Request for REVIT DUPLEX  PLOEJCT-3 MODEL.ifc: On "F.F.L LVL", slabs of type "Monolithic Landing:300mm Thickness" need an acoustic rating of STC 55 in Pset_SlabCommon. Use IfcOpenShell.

First a look at what the model holds.

```python
import ifcopenshell
import ifcopenshell.util.element

model = ifcopenshell.open("REVIT DUPLEX  PLOEJCT-3 MODEL.ifc")
print(model.schema)
storey = next(s for s in model.by_type("IfcBuildingStorey") if s.Name == "F.F.L LVL")
slabs = [e for e in ifcopenshell.util.element.get_decomposition(storey) if e.is_a("IfcSlab")]
seen = {}
for e in slabs:
    element_type = ifcopenshell.util.element.get_type(e)
    key = (element_type.Name if element_type != e and element_type else None, ifcopenshell.util.element.get_pset(e, "Pset_SlabCommon", "AcousticRating"))
    seen[key] = seen.get(key, 0) + 1
for (name, value), count in sorted(seen.items(), key=str):
    print(count, "x", name, "|", value)
```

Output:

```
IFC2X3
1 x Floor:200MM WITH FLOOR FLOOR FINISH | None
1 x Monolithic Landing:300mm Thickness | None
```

```python
import ifcopenshell
import ifcopenshell.api.pset
import ifcopenshell.util.element

model = ifcopenshell.open("REVIT DUPLEX  PLOEJCT-3 MODEL.ifc")

storey = next(s for s in model.by_type("IfcBuildingStorey") if s.Name == "F.F.L LVL")
slabs = [e for e in ifcopenshell.util.element.get_decomposition(storey) if e.is_a("IfcSlab")]

count = 0
for e in slabs:
    element_type = ifcopenshell.util.element.get_type(e)
    if element_type in (None, e) or element_type.Name != "Monolithic Landing:300mm Thickness":
        continue
    # add_pset returns the element's existing set when there is one.
    pset = ifcopenshell.api.pset.add_pset(model, product=e, name="Pset_SlabCommon")
    ifcopenshell.api.pset.edit_pset(model, pset=pset, properties={"AcousticRating": "STC 55"})
    count += 1

print(count, "slabs updated")

model.write("REVIT DUPLEX  PLOEJCT-3 MODEL-out.ifc")
```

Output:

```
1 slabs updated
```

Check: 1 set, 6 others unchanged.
